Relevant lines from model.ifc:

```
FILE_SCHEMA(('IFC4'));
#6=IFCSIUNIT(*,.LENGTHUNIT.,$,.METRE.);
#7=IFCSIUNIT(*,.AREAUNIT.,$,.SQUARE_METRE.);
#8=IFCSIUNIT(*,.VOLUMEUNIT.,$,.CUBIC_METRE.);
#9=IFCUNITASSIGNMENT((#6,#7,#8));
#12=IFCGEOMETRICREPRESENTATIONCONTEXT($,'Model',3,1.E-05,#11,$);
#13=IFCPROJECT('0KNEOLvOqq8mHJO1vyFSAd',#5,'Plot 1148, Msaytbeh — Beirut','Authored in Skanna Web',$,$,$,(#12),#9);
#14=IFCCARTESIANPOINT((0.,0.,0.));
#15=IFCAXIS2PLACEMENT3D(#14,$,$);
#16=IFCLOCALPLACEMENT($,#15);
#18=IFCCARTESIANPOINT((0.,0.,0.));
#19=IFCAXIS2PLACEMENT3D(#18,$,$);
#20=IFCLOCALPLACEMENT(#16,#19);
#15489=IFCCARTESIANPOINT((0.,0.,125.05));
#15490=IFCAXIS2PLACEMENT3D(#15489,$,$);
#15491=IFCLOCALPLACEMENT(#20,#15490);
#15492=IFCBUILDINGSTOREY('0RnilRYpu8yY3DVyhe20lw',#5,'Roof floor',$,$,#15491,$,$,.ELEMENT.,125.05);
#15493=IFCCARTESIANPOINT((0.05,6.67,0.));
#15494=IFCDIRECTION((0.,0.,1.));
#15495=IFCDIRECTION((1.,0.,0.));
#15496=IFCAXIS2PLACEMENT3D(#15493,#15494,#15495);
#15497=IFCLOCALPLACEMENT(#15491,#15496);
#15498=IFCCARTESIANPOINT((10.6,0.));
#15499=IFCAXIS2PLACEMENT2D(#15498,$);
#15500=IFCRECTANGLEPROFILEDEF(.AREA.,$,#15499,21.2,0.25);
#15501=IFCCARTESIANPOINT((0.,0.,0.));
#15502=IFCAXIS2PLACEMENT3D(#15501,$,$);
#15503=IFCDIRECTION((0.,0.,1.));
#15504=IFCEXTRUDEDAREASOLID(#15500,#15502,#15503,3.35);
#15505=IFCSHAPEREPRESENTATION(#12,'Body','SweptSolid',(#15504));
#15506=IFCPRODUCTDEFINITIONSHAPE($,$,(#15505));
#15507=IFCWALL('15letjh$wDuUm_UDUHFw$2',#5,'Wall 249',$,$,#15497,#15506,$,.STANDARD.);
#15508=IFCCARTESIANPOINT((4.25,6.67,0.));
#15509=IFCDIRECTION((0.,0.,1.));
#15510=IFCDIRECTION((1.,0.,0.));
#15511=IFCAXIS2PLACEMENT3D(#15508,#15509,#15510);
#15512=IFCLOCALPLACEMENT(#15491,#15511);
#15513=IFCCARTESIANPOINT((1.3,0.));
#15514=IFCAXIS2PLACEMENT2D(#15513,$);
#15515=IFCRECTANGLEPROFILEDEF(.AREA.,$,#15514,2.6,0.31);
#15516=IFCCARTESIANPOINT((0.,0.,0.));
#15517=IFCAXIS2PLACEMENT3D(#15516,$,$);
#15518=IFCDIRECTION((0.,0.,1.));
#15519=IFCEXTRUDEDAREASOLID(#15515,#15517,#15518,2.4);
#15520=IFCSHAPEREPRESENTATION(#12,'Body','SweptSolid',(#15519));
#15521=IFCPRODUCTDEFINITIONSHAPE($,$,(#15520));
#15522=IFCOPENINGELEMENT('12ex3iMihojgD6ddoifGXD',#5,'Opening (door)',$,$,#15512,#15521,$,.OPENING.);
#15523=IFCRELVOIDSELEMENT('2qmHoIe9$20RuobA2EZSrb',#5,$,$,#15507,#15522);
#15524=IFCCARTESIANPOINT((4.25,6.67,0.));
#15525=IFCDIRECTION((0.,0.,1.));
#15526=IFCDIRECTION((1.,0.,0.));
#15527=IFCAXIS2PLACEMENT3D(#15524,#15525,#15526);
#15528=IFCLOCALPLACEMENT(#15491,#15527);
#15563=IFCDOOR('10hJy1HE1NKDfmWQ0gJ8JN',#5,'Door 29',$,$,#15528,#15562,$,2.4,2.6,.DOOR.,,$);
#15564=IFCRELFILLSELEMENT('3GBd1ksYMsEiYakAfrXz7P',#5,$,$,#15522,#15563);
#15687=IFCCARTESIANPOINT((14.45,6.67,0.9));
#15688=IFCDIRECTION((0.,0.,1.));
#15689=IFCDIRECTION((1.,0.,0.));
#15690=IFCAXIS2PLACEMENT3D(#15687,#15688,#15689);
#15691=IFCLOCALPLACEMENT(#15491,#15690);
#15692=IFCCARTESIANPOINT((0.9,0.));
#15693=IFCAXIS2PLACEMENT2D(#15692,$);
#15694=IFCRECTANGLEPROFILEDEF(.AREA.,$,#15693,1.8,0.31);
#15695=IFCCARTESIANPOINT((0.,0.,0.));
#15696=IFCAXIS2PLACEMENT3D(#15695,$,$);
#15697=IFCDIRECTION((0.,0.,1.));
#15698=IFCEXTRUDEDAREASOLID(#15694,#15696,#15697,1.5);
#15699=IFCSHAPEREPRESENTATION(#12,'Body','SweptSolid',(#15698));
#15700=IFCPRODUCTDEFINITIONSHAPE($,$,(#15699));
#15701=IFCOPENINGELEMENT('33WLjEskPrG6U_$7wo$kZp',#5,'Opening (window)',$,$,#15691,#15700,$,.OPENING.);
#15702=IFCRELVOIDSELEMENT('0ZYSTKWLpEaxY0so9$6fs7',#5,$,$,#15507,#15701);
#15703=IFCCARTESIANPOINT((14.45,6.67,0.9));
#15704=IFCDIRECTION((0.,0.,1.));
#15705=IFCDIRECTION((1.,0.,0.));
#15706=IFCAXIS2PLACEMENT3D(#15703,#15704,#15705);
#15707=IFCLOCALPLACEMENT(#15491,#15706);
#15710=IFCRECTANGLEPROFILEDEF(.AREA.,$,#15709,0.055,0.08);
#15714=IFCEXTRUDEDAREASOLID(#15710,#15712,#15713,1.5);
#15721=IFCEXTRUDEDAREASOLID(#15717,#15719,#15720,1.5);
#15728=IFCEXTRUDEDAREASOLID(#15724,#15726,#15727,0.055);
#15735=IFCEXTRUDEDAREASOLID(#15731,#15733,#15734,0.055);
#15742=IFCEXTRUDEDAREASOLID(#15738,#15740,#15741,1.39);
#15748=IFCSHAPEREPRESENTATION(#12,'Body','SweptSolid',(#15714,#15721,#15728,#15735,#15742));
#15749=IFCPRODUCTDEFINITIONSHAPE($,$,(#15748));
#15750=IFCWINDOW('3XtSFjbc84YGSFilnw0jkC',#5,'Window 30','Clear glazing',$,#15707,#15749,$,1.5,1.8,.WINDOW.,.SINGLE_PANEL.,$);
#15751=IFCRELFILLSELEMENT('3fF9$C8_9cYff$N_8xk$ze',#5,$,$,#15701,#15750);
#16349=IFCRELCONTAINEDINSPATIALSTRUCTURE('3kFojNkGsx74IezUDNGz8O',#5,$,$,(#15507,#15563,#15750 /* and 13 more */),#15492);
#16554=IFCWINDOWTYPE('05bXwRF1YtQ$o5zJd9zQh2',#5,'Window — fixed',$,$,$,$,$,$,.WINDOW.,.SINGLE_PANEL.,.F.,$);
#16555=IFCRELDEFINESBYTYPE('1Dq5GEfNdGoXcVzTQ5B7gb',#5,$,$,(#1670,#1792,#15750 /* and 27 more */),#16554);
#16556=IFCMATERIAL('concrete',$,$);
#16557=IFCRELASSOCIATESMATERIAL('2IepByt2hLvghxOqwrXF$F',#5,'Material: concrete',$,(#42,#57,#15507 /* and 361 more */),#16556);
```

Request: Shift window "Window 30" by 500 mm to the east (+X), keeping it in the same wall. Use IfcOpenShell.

```python
import ifcopenshell
import ifcopenshell.api.geometry
import ifcopenshell.util.placement

model = ifcopenshell.open("model.ifc")

window = model.by_guid("3XtSFjbc84YGSFilnw0jkC")
opening = window.FillsVoids[0].RelatingOpeningElement
wall = opening.VoidsElements[0].RelatingBuildingElement

wall_matrix = ifcopenshell.util.placement.get_local_placement(wall.ObjectPlacement)
shift = wall_matrix[:3, 0] * 0.5
before = ifcopenshell.util.placement.get_local_placement(window.ObjectPlacement)[:3, 3].copy()

# The window is not placed relative to its opening, so move both.
for product in (opening, window):
    matrix = ifcopenshell.util.placement.get_local_placement(product.ObjectPlacement)
    matrix[:3, 3] += shift
    ifcopenshell.api.geometry.edit_object_placement(model, product=product, matrix=matrix, is_si=False)

after = ifcopenshell.util.placement.get_local_placement(window.ObjectPlacement)[:3, 3]
print("window moved by", (after - before).round(3) + 0.0)

model.write("model-out.ifc")
```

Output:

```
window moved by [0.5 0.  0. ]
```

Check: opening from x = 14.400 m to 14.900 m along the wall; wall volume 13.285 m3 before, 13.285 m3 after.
